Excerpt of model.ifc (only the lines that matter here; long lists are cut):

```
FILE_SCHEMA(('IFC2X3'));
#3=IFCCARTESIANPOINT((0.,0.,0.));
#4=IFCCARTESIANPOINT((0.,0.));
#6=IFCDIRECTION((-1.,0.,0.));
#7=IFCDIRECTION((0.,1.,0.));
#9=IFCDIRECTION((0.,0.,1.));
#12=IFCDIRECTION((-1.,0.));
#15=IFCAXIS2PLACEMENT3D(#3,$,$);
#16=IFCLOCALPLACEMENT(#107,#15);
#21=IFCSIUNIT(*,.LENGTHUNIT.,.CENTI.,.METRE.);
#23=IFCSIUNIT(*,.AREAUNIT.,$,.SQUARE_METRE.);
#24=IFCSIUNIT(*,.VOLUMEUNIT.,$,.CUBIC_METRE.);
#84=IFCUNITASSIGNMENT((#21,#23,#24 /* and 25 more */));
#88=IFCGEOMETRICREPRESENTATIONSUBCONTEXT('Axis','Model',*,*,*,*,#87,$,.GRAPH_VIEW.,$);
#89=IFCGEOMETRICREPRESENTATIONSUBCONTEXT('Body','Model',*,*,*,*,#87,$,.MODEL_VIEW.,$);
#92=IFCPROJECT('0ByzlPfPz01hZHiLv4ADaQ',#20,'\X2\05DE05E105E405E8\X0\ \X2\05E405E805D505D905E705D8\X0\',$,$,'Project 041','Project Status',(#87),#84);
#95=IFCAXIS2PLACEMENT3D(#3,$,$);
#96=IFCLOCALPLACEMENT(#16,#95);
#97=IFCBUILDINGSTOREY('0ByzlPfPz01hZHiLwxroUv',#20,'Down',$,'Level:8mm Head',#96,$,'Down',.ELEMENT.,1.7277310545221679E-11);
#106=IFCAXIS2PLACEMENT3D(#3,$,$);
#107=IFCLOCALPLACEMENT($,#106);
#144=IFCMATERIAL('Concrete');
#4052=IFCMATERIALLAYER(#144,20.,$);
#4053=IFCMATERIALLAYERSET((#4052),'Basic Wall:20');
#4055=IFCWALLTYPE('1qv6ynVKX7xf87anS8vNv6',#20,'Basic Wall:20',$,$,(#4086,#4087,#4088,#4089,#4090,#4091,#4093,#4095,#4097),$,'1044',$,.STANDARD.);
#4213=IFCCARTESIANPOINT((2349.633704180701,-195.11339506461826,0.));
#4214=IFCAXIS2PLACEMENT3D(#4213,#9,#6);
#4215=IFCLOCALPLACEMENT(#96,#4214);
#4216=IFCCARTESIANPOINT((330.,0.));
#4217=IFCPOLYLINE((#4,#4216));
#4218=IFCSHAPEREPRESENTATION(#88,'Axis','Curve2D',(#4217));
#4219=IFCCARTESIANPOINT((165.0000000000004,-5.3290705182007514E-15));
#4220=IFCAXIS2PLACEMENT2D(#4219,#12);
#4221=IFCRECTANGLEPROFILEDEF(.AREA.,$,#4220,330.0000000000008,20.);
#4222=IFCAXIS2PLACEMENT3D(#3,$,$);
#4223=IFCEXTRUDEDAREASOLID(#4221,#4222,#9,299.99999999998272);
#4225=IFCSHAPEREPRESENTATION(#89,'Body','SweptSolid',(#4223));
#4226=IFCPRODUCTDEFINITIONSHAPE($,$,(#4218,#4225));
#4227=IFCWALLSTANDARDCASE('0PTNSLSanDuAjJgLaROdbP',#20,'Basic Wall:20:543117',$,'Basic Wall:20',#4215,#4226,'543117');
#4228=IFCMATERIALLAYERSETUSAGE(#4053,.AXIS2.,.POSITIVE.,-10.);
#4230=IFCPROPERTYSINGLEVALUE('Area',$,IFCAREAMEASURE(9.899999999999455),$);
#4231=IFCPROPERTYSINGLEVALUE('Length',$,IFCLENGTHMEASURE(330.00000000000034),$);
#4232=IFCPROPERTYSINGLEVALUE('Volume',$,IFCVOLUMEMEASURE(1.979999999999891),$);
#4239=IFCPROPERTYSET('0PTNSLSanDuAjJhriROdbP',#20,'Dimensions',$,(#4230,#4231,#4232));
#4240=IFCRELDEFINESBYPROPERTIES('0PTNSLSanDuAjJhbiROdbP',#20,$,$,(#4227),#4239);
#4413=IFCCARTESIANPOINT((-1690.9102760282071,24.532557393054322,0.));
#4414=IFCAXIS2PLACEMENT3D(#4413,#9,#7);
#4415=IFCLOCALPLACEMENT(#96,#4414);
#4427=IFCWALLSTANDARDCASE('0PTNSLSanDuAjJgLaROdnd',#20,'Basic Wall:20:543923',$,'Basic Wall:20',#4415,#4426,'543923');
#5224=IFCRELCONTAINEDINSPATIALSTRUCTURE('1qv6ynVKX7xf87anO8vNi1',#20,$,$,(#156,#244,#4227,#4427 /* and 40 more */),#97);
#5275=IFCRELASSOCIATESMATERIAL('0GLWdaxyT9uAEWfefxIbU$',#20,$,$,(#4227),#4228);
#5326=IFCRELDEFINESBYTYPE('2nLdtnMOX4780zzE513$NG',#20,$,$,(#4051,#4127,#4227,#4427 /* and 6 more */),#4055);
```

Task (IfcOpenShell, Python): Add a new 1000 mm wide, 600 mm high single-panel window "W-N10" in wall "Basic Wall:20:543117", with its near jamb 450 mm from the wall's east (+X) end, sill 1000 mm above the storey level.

```python
import numpy as np
import ifcopenshell
import ifcopenshell.api.feature
import ifcopenshell.api.geometry
import ifcopenshell.api.pset
import ifcopenshell.api.root
import ifcopenshell.api.spatial
import ifcopenshell.api.type
import ifcopenshell.geom
import ifcopenshell.util.element
import ifcopenshell.util.placement
import ifcopenshell.util.representation
import ifcopenshell.util.shape
import ifcopenshell.util.unit

model = ifcopenshell.open("model.ifc")
unit_scale = ifcopenshell.util.unit.calculate_unit_scale(model)
area_scale = ifcopenshell.util.unit.calculate_unit_scale(model, "AREAUNIT")
volume_scale = ifcopenshell.util.unit.calculate_unit_scale(model, "VOLUMEUNIT")
settings = ifcopenshell.geom.settings()


def volume(element):
    """Net volume in cubic metres, openings subtracted."""
    shape = ifcopenshell.geom.create_shape(settings, element)
    return ifcopenshell.util.shape.get_volume(shape.geometry)


wall = model.by_guid("0PTNSLSanDuAjJgLaROdbP")
storey = ifcopenshell.util.element.get_container(wall, ifc_class="IfcBuildingStorey")
context = ifcopenshell.util.representation.get_context(model, "Model", "Body", "MODEL_VIEW")
before = volume(wall)

width, height, from_end, sill = 1, 0.6, 0.45, 1  # metres

# The wall runs along its own X axis, and the end named is its -X end.
wall_shape = ifcopenshell.geom.create_shape(settings, wall)
x, y, z = ifcopenshell.util.shape.get_vertices(wall_shape.geometry).T
start = x.min() + from_end
face, thickness = float(y.min()), float(y.max() - y.min())
wall_matrix = ifcopenshell.util.placement.get_local_placement(wall.ObjectPlacement)
level = ifcopenshell.util.placement.get_local_placement(storey.ObjectPlacement)[2, 3]


def in_wall(x, y):
    """Placement at x, y metres in the wall's axes, at sill height."""
    matrix = wall_matrix.copy()
    matrix[:, 3] = wall_matrix @ np.array([x / unit_scale, y / unit_scale, 0.0, 1.0])
    matrix[2, 3] = level + sill / unit_scale
    return matrix


# Opening: a box that overshoots both wall faces by 50 mm.
opening = ifcopenshell.api.root.create_entity(model, ifc_class="IfcOpeningElement")
box = ifcopenshell.api.geometry.add_wall_representation(
    model, context=context, length=width, height=height, thickness=thickness + 0.1
)
ifcopenshell.api.geometry.assign_representation(model, product=opening, representation=box)
ifcopenshell.api.geometry.edit_object_placement(model, product=opening, matrix=in_wall(start, face - 0.05), is_si=False)
ifcopenshell.api.feature.add_feature(model, feature=opening, element=wall)

window = ifcopenshell.api.root.create_entity(model, ifc_class="IfcWindow", name="W-N10")
window.OverallWidth, window.OverallHeight = width / unit_scale, height / unit_scale
body = ifcopenshell.api.geometry.add_window_representation(
    model,
    context=context,
    overall_width=window.OverallWidth,
    overall_height=window.OverallHeight,
    partition_type="SINGLE_PANEL",
)
ifcopenshell.api.geometry.assign_representation(model, product=window, representation=body)
ifcopenshell.api.spatial.assign_container(model, products=[window], relating_structure=storey)
fills = ifcopenshell.api.feature.add_filling(model, opening=opening, element=window)
fills.OwnerHistory = window.OwnerHistory  # required in IFC2X3

# IFC2X3 keeps the operation on the window style.
style = ifcopenshell.api.root.create_entity(model, ifc_class="IfcWindowStyle", name="W-N10")
style.OperationType, style.ConstructionType = "SINGLE_PANEL", "NOTDEFINED"
style.ParameterTakesPrecedence = style.Sizeable = False
ifcopenshell.api.type.assign_type(model, related_objects=[window], relating_type=style)

# Centre the window in the wall's thickness.
ifcopenshell.api.geometry.edit_object_placement(model, product=window, matrix=in_wall(start, face), is_si=False)
window_shape = ifcopenshell.geom.create_shape(settings, window)
depth = ifcopenshell.util.shape.get_vertices(window_shape.geometry)[:, 1]
offset = face + thickness / 2 - (depth.min() + depth.max()) / 2
ifcopenshell.api.geometry.edit_object_placement(model, product=window, matrix=in_wall(start, offset), is_si=False)

after = volume(wall)

# Update the wall's stored quantities.
pset = model.by_id(ifcopenshell.util.element.get_pset(wall, "Dimensions", should_inherit=False)["id"])
ifcopenshell.api.pset.edit_pset(model, pset=pset, properties={
    "Area": model.create_entity("IfcAreaMeasure", after / thickness / area_scale),
    "Volume": model.create_entity("IfcVolumeMeasure", after / volume_scale),
})

print(f"wall volume {before:.3f} -> {after:.3f} m3")

model.write("model_rev.ifc")
```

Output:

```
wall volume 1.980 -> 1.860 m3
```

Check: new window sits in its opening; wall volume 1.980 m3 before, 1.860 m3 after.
